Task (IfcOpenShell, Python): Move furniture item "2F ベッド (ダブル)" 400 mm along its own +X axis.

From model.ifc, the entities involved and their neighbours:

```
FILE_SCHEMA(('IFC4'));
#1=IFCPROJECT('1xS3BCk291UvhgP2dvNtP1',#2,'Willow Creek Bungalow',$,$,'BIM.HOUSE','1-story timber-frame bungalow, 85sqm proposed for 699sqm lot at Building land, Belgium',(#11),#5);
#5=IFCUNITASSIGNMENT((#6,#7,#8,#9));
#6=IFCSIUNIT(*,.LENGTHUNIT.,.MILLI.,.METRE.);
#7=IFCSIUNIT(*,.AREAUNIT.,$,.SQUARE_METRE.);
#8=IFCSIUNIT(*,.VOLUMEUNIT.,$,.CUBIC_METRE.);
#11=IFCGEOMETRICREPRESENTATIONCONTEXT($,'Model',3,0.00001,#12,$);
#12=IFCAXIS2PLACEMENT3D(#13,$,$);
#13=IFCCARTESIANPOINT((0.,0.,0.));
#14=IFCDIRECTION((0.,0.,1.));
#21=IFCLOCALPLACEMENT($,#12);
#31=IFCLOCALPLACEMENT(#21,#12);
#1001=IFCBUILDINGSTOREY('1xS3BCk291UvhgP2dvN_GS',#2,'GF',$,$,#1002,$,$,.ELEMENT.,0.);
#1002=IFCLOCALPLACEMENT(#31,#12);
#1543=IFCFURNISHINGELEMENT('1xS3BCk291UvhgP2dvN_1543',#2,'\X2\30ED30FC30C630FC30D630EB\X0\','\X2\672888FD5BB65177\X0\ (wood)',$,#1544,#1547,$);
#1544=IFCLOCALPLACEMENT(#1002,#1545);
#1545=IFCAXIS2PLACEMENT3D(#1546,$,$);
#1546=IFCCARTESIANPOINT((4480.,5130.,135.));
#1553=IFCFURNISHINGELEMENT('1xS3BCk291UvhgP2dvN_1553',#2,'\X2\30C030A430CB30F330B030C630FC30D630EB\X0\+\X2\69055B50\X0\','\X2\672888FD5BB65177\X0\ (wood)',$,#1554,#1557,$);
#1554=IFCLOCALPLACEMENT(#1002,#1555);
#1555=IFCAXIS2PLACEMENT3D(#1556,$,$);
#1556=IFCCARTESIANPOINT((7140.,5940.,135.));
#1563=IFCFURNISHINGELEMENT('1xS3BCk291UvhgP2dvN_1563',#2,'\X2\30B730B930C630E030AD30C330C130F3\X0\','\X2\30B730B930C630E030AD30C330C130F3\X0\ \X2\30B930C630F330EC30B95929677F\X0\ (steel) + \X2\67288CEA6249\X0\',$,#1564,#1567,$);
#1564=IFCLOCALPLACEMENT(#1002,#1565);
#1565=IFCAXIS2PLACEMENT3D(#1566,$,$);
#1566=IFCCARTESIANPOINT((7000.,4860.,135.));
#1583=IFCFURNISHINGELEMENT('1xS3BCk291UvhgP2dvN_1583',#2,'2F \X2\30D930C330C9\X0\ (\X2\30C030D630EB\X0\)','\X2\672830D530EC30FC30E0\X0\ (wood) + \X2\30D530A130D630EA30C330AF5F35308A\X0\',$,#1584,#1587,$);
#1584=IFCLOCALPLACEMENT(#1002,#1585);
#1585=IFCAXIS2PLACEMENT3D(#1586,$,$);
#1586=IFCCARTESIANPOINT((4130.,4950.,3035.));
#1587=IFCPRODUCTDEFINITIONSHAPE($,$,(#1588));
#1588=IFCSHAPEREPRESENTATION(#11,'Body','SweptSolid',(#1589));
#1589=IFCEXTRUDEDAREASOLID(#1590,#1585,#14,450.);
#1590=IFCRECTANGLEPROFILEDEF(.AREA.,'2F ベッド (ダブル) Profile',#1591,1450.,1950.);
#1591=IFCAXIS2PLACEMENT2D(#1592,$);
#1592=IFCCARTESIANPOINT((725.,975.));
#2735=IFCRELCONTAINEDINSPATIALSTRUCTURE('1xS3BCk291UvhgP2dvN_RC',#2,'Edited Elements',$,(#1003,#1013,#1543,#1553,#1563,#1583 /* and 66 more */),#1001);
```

```python
import ifcopenshell
import ifcopenshell.api.geometry
import ifcopenshell.util.placement

model = ifcopenshell.open("model.ifc")

item = model.by_guid("1xS3BCk291UvhgP2dvN_1583")
matrix = ifcopenshell.util.placement.get_local_placement(item.ObjectPlacement)
matrix[:3, 3] += matrix[:3, 0] * 400.0
ifcopenshell.api.geometry.edit_object_placement(model, product=item, matrix=matrix, is_si=False)

print(ifcopenshell.util.placement.get_local_placement(item.ObjectPlacement).round(3) + 0.0)

model.write("model_rev.ifc")
```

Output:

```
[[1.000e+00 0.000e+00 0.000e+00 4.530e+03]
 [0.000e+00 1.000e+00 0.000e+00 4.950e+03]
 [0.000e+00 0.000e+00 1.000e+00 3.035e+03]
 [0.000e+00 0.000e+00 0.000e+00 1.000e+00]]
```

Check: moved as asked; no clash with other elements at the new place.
